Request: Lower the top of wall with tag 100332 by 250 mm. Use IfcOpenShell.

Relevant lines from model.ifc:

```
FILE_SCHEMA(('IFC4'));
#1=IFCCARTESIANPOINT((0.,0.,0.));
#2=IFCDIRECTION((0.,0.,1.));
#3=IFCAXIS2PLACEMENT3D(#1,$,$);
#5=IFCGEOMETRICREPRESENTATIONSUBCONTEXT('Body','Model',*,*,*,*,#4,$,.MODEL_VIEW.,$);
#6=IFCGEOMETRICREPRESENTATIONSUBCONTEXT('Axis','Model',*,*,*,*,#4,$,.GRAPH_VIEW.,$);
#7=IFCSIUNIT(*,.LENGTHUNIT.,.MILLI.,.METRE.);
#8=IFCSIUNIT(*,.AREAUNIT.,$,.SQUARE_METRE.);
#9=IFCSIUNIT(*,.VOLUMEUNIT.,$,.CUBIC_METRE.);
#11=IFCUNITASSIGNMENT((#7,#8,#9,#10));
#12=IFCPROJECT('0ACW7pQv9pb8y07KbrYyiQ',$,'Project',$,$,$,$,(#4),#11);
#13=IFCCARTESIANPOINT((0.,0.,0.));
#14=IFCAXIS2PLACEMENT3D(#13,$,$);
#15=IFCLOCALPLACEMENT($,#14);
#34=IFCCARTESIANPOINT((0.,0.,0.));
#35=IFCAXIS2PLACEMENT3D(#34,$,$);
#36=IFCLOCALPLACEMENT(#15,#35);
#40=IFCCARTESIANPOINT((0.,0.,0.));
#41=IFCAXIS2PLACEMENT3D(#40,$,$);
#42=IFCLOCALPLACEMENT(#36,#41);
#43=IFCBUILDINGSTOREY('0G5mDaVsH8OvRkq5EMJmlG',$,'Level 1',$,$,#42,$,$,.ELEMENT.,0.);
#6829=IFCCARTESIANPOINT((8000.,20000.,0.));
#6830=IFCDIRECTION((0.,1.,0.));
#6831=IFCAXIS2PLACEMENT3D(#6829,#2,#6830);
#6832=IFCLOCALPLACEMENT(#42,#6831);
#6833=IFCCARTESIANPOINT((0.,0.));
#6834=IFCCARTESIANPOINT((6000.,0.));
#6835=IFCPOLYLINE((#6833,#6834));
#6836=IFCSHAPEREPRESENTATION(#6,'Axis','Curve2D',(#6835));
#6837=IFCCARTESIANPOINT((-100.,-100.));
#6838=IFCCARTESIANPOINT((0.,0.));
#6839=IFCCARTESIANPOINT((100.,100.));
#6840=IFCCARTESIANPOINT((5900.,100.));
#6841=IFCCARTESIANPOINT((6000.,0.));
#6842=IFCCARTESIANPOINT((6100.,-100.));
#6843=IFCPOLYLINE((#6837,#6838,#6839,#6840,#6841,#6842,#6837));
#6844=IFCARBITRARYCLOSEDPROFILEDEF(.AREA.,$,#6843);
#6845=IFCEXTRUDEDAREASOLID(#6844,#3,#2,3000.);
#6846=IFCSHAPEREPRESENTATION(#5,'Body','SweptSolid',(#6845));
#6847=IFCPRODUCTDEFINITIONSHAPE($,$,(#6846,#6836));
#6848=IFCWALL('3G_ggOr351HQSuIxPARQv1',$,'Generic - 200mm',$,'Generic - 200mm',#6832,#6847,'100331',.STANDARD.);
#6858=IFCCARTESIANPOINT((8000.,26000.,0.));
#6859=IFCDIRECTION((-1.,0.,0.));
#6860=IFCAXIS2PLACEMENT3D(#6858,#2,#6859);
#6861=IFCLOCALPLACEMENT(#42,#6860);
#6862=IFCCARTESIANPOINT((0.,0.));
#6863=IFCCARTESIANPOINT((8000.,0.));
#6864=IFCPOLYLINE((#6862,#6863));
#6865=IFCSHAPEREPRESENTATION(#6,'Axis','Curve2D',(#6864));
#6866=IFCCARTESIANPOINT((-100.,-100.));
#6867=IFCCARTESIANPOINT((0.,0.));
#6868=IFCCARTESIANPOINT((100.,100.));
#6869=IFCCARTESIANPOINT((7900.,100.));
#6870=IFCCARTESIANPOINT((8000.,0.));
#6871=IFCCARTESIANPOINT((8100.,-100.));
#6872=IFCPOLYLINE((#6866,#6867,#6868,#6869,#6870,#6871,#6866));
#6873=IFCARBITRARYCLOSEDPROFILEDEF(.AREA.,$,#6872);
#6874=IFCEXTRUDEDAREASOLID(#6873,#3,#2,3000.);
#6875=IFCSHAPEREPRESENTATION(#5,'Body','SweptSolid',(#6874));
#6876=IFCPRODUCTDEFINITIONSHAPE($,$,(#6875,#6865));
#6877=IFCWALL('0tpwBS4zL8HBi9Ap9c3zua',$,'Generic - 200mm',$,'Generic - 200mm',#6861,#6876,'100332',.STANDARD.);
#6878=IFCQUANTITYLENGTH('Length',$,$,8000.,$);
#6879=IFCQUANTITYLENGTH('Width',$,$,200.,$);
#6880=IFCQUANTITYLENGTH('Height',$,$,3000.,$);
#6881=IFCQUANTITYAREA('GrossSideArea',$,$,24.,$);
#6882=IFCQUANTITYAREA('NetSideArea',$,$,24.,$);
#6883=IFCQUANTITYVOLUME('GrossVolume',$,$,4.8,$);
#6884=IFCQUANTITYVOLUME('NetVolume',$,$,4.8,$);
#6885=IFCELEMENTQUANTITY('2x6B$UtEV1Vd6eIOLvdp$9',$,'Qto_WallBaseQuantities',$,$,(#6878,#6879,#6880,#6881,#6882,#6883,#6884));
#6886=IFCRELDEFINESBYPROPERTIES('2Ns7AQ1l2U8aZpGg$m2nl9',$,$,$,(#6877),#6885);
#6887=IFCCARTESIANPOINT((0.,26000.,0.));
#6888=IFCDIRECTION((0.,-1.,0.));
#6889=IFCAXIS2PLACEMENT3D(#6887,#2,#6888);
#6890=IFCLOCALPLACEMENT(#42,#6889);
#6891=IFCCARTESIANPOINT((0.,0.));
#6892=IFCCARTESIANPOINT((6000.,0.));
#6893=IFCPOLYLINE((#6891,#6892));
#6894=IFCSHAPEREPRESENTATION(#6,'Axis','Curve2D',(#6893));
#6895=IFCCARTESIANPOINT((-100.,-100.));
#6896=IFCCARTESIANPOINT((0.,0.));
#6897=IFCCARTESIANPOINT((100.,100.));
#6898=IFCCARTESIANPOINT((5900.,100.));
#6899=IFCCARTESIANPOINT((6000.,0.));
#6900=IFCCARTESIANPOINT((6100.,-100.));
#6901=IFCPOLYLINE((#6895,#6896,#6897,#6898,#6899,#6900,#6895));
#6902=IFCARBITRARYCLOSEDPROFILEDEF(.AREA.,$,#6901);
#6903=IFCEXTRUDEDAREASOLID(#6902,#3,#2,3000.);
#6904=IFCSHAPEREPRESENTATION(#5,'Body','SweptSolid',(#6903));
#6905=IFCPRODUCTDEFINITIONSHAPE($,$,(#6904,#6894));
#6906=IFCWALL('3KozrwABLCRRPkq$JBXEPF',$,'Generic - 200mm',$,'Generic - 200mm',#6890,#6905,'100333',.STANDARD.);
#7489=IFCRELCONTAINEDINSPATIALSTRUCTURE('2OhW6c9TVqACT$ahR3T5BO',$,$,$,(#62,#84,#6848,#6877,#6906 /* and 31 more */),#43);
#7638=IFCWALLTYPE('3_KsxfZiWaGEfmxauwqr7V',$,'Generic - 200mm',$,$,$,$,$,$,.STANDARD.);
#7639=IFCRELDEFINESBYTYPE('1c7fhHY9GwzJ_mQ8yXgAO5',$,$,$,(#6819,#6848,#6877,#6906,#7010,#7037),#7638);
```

```python
import ifcopenshell
import ifcopenshell.api.pset
import ifcopenshell.geom
import ifcopenshell.util.element
import ifcopenshell.util.representation
import ifcopenshell.util.shape
import ifcopenshell.util.unit

model = ifcopenshell.open("model.ifc")
unit_scale = ifcopenshell.util.unit.calculate_unit_scale(model)
area_scale = ifcopenshell.util.unit.calculate_unit_scale(model, "AREAUNIT")
volume_scale = ifcopenshell.util.unit.calculate_unit_scale(model, "VOLUMEUNIT")
settings = ifcopenshell.geom.settings()


def volume(element):
    """Net volume in cubic metres, openings subtracted."""
    shape = ifcopenshell.geom.create_shape(settings, element)
    return ifcopenshell.util.shape.get_volume(shape.geometry)


wall = model.by_guid("0tpwBS4zL8HBi9Ap9c3zua")
before = volume(wall)

body = ifcopenshell.util.representation.get_representation(wall, "Model", "Body")
solid = body.Items[0]
old_height = solid.Depth
solid.Depth -= 0.25 / unit_scale
after = volume(wall)
thickness = 0.2  # wall thickness in metres

# Update the stored height, areas and volumes.
qto = model.by_id(ifcopenshell.util.element.get_pset(wall, "Qto_WallBaseQuantities", should_inherit=False)["id"])
ifcopenshell.api.pset.edit_qto(model, qto=qto, properties={
    "Height": solid.Depth,
    "GrossSideArea": ifcopenshell.util.element.get_pset(wall, "Qto_WallBaseQuantities", "GrossSideArea") * solid.Depth / old_height,
    "NetSideArea": after / thickness / area_scale,
    "GrossVolume": ifcopenshell.util.element.get_pset(wall, "Qto_WallBaseQuantities", "GrossVolume") * solid.Depth / old_height,
    "NetVolume": after / volume_scale,
})

print(f"height {old_height:g} -> {solid.Depth:g}, volume {before:.3f} -> {after:.3f} m3")

model.write("model-out.ifc")
```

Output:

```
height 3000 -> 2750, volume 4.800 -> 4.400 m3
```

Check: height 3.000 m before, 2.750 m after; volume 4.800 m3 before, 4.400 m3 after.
